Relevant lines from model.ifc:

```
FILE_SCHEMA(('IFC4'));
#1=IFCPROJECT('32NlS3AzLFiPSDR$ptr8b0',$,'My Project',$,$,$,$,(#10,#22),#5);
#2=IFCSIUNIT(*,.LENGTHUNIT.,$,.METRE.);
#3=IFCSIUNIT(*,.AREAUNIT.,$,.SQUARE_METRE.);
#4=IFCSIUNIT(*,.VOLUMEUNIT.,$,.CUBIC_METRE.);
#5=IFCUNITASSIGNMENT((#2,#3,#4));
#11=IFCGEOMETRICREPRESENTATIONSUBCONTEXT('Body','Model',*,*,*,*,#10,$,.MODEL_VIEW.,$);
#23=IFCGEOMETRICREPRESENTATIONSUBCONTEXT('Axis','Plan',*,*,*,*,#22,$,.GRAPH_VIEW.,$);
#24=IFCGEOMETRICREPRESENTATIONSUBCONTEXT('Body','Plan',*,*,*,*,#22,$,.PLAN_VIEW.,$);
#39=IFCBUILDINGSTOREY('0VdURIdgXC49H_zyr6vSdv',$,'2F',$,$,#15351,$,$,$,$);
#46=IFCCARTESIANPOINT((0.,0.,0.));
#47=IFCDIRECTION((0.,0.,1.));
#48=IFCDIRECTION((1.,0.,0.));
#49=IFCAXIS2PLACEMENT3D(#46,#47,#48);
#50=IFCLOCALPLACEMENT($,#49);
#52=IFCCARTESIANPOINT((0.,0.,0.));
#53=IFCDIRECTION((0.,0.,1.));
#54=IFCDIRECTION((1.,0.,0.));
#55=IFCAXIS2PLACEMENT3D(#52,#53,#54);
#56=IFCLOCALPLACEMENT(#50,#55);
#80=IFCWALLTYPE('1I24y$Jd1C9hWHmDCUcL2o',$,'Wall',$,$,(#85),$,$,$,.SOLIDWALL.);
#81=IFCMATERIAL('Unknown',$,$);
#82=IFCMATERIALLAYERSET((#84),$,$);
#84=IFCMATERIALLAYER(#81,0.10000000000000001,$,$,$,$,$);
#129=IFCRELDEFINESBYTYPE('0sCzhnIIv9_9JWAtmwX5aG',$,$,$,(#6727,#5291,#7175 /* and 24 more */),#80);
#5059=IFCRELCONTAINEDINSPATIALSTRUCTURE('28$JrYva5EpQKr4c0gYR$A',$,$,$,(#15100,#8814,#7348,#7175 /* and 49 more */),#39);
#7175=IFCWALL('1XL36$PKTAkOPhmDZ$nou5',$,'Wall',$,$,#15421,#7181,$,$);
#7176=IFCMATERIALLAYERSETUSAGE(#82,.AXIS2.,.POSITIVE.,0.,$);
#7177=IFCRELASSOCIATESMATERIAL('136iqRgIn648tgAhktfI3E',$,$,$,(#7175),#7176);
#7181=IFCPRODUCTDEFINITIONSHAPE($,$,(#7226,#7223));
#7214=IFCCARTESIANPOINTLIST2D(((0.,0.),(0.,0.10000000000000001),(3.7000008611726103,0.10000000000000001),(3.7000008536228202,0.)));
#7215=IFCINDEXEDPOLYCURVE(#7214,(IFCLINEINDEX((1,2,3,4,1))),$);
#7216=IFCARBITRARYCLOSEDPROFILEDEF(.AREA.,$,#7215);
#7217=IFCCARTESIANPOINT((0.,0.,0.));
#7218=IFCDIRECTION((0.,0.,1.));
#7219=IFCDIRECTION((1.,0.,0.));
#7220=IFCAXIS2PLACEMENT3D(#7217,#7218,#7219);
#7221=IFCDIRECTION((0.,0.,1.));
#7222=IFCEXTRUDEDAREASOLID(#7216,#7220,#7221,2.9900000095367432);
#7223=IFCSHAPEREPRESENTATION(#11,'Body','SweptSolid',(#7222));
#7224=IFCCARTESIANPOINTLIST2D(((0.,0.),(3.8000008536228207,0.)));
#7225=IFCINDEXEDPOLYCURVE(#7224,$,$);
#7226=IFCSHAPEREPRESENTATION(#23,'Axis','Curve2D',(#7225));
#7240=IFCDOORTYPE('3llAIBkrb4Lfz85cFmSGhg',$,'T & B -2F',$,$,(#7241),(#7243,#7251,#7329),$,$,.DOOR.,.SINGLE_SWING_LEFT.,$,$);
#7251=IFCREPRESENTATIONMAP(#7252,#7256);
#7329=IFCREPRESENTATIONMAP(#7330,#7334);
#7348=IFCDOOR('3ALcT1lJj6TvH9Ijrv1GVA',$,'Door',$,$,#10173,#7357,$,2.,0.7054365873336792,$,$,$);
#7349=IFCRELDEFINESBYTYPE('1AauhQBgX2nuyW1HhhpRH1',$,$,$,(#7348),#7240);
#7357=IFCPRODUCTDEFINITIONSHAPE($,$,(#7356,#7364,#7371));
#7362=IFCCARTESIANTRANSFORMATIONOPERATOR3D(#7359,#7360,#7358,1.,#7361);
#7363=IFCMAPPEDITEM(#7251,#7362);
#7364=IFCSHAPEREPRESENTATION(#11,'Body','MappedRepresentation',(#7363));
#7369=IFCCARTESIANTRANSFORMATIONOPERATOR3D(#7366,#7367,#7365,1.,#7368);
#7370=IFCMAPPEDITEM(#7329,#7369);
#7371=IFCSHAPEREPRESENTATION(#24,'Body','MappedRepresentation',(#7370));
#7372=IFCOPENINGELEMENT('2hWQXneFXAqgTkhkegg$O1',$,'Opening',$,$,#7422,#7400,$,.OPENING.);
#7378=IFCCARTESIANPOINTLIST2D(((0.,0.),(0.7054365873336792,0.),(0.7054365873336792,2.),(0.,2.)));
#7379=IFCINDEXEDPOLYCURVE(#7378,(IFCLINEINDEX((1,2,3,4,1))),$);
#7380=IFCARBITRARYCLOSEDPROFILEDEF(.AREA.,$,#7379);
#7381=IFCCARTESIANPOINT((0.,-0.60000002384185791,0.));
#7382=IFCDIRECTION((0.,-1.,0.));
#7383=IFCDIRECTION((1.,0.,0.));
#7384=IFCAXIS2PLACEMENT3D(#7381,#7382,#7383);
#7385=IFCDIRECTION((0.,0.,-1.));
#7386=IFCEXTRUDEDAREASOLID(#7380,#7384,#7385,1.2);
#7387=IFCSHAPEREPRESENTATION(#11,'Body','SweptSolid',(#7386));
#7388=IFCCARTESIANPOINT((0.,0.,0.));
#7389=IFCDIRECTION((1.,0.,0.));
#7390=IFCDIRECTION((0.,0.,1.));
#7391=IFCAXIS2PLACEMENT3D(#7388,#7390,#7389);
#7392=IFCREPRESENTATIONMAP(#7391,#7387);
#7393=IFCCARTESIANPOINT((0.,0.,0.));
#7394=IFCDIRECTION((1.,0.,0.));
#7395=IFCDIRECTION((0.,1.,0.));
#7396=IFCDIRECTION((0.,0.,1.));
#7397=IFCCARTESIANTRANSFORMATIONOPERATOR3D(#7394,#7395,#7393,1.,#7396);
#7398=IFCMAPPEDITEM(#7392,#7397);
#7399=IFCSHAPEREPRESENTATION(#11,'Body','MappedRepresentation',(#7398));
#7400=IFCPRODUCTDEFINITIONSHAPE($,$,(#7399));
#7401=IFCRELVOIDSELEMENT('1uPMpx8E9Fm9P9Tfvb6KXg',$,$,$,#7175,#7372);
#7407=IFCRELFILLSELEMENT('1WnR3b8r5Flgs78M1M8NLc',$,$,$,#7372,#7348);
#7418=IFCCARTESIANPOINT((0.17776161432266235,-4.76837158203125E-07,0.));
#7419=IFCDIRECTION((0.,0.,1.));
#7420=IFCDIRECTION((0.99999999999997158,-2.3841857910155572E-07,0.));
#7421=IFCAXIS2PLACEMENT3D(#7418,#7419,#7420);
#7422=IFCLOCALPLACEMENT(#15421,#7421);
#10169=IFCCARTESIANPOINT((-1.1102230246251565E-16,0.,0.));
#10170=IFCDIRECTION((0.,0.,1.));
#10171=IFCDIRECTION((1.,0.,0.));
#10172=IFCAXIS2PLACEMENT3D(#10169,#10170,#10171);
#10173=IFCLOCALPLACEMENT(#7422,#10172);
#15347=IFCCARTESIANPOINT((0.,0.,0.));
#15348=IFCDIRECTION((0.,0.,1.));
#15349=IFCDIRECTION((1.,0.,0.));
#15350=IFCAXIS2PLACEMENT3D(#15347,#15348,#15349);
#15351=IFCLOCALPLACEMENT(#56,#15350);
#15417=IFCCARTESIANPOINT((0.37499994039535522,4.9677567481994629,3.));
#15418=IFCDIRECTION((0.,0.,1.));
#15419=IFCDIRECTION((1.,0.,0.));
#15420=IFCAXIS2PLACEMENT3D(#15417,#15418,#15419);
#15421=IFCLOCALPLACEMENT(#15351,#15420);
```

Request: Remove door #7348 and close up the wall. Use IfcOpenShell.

```python
import ifcopenshell
import ifcopenshell.api.feature
import ifcopenshell.api.root
import ifcopenshell.geom
import ifcopenshell.util.shape

model = ifcopenshell.open("model.ifc")
settings = ifcopenshell.geom.settings()


def volume(element):
    """Net volume in cubic metres, openings subtracted."""
    shape = ifcopenshell.geom.create_shape(settings, element)
    return ifcopenshell.util.shape.get_volume(shape.geometry)


door = model.by_guid("3ALcT1lJj6TvH9Ijrv1GVA")
opening = door.FillsVoids[0].RelatingOpeningElement
wall = opening.VoidsElements[0].RelatingBuildingElement
before = volume(wall)

ifcopenshell.api.root.remove_product(model, product=door)
ifcopenshell.api.feature.remove_feature(model, feature=opening)

after = volume(wall)

print(f"wall volume {before:.3f} -> {after:.3f} m3")

model.write("model_rev.ifc")
```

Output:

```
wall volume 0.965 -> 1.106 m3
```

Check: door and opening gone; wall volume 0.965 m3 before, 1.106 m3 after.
